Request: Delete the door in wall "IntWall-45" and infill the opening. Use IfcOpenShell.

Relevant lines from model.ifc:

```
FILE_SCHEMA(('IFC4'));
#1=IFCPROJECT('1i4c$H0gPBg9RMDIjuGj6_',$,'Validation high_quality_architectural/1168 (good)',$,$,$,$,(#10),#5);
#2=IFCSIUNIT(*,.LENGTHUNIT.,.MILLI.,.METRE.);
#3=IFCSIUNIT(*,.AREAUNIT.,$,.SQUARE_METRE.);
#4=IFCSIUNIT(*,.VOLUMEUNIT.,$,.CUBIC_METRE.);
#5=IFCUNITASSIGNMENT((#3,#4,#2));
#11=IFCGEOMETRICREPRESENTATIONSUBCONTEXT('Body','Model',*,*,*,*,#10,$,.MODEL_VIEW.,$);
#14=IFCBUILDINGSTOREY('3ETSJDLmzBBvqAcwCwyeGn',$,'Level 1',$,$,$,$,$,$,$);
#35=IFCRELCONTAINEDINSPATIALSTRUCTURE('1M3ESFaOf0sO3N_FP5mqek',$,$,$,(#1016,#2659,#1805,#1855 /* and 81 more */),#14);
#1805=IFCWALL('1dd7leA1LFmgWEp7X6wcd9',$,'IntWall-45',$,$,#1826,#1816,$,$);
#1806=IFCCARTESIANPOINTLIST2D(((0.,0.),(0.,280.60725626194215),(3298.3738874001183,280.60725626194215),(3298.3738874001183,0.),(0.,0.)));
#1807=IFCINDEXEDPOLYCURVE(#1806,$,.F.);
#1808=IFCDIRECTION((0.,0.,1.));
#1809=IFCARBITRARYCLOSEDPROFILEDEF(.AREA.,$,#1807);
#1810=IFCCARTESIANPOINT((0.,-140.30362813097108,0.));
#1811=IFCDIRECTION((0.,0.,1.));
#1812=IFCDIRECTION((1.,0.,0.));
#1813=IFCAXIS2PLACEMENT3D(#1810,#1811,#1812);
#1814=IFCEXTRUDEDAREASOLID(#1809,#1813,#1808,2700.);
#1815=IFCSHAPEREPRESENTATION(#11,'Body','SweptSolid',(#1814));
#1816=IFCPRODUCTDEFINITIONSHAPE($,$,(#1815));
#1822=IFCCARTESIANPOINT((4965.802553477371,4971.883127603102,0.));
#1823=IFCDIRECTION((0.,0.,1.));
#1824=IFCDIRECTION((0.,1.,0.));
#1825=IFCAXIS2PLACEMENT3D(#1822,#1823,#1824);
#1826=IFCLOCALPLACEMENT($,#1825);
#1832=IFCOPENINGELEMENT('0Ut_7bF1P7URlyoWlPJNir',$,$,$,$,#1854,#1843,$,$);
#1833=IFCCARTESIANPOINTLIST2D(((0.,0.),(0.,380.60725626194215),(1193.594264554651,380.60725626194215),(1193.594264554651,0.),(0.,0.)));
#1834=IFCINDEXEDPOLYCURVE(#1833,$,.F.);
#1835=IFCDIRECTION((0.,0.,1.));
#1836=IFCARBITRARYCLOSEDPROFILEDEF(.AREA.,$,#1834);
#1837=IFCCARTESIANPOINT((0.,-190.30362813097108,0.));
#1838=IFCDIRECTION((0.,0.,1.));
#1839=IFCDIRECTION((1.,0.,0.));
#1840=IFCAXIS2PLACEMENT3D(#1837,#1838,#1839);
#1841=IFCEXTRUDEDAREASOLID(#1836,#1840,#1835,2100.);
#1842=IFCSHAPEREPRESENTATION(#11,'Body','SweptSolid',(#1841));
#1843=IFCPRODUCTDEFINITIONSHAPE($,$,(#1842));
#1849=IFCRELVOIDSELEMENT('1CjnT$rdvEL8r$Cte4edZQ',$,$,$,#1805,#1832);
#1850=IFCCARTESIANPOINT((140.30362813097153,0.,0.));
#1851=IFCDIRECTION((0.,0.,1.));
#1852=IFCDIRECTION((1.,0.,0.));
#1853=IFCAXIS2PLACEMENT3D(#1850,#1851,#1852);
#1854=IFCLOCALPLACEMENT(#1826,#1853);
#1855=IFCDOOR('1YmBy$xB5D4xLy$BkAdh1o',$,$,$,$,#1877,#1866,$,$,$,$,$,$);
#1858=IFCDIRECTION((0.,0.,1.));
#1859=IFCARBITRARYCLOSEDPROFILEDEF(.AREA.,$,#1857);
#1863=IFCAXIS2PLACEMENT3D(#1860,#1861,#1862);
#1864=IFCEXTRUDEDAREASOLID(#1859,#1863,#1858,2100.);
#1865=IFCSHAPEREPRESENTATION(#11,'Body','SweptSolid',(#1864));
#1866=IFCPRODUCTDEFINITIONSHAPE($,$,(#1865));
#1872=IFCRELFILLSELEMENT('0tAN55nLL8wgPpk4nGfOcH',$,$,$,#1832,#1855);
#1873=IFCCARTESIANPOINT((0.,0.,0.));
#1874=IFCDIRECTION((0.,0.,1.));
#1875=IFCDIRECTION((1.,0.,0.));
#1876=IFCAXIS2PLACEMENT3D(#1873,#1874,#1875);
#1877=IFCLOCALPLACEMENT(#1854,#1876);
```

```python
import ifcopenshell
import ifcopenshell.api.feature
import ifcopenshell.api.root
import ifcopenshell.geom
import ifcopenshell.util.shape

model = ifcopenshell.open("model.ifc")
settings = ifcopenshell.geom.settings()


def volume(element):
    """Net volume in cubic metres, openings subtracted."""
    shape = ifcopenshell.geom.create_shape(settings, element)
    return ifcopenshell.util.shape.get_volume(shape.geometry)


door = model.by_id(1855)
opening = door.FillsVoids[0].RelatingOpeningElement
wall = opening.VoidsElements[0].RelatingBuildingElement
before = volume(wall)

ifcopenshell.api.root.remove_product(model, product=door)
ifcopenshell.api.feature.remove_feature(model, feature=opening)

after = volume(wall)

print(f"wall volume {before:.3f} -> {after:.3f} m3")

model.write("model_rev.ifc")
```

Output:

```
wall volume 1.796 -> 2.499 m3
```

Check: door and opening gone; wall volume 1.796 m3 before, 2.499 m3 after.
